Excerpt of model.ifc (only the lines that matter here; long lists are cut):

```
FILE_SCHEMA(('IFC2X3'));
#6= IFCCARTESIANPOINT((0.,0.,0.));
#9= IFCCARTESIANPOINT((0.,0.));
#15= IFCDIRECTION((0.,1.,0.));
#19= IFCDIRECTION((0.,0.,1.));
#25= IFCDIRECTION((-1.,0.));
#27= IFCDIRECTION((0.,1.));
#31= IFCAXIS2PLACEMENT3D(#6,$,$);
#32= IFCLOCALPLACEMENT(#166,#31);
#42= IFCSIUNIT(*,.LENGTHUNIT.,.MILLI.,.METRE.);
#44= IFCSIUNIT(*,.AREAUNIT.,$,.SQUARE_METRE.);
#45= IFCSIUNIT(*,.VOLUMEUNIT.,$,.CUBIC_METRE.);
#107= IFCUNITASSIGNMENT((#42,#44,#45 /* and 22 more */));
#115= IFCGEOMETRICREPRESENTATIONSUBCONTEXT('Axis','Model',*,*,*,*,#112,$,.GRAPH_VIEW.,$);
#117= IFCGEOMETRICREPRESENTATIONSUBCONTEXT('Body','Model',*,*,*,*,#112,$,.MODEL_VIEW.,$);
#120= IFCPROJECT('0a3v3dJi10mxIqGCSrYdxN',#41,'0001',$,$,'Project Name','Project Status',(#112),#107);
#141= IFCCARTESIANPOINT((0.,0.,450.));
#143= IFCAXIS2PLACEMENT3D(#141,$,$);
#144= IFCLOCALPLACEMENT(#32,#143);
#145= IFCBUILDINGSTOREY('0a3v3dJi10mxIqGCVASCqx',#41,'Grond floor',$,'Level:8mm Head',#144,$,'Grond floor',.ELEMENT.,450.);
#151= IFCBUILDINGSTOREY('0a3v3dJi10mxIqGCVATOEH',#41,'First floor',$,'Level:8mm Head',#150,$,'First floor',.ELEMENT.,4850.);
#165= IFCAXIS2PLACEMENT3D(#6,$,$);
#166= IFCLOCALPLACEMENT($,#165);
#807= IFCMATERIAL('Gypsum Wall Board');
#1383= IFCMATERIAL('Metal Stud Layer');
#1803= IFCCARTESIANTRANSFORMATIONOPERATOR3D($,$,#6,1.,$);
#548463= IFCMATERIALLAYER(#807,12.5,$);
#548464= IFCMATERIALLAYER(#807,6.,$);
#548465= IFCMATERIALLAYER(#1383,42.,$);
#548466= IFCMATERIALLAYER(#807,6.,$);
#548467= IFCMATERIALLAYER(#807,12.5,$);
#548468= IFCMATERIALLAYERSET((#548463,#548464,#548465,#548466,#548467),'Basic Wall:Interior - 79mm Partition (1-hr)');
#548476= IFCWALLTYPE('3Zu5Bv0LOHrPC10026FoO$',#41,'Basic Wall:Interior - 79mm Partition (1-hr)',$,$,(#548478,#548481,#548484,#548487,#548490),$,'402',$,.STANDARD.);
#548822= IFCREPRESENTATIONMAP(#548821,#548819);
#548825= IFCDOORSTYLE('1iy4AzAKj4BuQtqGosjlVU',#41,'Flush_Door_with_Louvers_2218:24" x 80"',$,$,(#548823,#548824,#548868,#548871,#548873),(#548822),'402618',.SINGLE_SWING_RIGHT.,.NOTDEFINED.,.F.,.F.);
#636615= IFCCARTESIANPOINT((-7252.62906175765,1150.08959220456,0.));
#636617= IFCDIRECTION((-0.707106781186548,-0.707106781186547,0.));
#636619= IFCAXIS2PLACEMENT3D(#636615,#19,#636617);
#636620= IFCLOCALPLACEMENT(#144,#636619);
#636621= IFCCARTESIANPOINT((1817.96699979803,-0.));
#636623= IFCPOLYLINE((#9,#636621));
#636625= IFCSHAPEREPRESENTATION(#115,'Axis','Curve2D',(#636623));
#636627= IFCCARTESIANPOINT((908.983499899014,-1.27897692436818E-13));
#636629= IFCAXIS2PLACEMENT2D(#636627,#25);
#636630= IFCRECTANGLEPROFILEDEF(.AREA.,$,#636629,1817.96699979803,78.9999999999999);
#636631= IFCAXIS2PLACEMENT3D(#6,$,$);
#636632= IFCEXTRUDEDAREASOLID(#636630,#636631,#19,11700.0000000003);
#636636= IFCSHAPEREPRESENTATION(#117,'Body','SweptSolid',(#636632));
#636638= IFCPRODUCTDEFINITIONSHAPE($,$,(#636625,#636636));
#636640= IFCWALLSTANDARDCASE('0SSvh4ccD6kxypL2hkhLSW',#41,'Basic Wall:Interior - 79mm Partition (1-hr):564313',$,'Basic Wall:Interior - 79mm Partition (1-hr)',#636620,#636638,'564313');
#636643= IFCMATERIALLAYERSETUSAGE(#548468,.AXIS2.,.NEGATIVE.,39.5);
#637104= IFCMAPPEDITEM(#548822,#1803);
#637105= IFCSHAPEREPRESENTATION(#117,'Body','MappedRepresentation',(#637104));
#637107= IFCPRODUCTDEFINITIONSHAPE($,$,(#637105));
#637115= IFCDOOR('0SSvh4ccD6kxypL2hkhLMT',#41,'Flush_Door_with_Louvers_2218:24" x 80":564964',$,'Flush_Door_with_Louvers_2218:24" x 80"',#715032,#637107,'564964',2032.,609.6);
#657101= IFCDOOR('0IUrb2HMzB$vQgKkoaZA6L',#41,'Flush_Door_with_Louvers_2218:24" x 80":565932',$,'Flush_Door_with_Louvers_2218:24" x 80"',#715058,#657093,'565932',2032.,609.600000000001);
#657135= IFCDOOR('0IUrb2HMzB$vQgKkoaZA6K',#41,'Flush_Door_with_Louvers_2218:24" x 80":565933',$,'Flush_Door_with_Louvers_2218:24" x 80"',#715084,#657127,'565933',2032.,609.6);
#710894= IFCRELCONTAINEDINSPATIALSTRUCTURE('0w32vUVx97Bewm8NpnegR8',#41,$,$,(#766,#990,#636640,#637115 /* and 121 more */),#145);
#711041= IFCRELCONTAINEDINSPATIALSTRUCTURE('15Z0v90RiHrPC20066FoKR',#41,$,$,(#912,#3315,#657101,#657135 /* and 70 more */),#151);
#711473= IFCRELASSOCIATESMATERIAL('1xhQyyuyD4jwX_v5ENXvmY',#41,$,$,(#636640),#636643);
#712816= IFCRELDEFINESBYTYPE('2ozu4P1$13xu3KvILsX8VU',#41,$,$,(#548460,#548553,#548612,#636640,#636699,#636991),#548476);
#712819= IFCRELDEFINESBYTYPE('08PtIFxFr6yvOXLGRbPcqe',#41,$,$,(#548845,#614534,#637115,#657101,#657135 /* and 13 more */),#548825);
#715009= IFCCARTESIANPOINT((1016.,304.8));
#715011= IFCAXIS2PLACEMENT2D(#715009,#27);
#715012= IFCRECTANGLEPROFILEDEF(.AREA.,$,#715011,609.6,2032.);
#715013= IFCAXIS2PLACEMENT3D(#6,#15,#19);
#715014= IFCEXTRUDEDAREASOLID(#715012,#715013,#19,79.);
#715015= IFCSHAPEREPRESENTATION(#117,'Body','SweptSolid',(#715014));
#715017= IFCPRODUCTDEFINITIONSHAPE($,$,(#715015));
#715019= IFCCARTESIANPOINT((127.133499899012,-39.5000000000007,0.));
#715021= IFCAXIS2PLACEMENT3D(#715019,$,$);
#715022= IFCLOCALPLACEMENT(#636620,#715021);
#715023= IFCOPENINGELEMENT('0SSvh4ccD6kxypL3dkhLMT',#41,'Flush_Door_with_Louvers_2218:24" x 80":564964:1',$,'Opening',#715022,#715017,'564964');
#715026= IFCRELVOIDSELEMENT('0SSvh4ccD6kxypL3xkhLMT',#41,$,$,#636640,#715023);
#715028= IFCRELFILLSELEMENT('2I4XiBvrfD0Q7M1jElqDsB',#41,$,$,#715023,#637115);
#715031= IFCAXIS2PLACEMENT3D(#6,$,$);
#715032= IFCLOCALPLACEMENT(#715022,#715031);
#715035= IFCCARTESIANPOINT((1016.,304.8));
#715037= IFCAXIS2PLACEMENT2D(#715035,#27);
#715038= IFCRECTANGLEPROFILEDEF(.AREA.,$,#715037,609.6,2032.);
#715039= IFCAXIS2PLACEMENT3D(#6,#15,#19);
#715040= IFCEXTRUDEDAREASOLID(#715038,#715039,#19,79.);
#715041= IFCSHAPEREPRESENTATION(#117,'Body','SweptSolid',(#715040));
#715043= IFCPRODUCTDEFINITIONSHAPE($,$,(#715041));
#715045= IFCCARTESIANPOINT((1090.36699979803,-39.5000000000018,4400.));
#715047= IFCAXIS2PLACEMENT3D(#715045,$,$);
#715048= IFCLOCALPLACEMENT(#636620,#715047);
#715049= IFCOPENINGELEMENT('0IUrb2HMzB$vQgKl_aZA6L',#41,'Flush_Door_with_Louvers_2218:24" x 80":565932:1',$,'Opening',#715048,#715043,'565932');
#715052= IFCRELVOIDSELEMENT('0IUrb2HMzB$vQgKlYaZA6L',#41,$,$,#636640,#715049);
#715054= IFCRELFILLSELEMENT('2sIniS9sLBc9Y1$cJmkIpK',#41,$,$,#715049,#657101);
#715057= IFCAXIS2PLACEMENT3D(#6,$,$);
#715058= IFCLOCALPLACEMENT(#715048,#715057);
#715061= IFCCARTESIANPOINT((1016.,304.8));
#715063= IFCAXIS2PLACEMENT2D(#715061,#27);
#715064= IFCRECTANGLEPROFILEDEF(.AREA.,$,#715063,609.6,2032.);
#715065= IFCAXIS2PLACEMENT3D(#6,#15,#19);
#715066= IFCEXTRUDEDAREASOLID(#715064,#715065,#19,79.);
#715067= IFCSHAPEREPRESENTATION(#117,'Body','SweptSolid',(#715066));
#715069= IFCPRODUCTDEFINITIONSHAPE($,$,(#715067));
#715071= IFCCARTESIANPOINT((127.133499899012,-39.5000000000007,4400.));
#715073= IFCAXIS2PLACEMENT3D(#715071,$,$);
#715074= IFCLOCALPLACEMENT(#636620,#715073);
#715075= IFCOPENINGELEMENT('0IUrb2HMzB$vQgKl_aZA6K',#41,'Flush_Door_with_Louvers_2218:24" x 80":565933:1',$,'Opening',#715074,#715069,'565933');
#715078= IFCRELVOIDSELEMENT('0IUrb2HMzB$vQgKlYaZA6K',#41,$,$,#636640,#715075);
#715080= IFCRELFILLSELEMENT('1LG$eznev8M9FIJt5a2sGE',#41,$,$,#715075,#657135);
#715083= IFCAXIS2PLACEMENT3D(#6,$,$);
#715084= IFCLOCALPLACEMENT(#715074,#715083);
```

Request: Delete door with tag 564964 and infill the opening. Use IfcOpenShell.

```python
import ifcopenshell
import ifcopenshell.api.feature
import ifcopenshell.api.root
import ifcopenshell.geom
import ifcopenshell.util.shape

model = ifcopenshell.open("model.ifc")
settings = ifcopenshell.geom.settings()


def volume(element):
    """Net volume in cubic metres, openings subtracted."""
    shape = ifcopenshell.geom.create_shape(settings, element)
    return ifcopenshell.util.shape.get_volume(shape.geometry)


door = model.by_guid("0SSvh4ccD6kxypL2hkhLMT")
opening = door.FillsVoids[0].RelatingOpeningElement
wall = opening.VoidsElements[0].RelatingBuildingElement
before = volume(wall)

ifcopenshell.api.root.remove_product(model, product=door)
ifcopenshell.api.feature.remove_feature(model, feature=opening)

after = volume(wall)

print(f"wall volume {before:.3f} -> {after:.3f} m3")

model.write("model-out.ifc")
```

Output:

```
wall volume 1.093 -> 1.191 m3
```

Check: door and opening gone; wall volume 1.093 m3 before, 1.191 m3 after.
